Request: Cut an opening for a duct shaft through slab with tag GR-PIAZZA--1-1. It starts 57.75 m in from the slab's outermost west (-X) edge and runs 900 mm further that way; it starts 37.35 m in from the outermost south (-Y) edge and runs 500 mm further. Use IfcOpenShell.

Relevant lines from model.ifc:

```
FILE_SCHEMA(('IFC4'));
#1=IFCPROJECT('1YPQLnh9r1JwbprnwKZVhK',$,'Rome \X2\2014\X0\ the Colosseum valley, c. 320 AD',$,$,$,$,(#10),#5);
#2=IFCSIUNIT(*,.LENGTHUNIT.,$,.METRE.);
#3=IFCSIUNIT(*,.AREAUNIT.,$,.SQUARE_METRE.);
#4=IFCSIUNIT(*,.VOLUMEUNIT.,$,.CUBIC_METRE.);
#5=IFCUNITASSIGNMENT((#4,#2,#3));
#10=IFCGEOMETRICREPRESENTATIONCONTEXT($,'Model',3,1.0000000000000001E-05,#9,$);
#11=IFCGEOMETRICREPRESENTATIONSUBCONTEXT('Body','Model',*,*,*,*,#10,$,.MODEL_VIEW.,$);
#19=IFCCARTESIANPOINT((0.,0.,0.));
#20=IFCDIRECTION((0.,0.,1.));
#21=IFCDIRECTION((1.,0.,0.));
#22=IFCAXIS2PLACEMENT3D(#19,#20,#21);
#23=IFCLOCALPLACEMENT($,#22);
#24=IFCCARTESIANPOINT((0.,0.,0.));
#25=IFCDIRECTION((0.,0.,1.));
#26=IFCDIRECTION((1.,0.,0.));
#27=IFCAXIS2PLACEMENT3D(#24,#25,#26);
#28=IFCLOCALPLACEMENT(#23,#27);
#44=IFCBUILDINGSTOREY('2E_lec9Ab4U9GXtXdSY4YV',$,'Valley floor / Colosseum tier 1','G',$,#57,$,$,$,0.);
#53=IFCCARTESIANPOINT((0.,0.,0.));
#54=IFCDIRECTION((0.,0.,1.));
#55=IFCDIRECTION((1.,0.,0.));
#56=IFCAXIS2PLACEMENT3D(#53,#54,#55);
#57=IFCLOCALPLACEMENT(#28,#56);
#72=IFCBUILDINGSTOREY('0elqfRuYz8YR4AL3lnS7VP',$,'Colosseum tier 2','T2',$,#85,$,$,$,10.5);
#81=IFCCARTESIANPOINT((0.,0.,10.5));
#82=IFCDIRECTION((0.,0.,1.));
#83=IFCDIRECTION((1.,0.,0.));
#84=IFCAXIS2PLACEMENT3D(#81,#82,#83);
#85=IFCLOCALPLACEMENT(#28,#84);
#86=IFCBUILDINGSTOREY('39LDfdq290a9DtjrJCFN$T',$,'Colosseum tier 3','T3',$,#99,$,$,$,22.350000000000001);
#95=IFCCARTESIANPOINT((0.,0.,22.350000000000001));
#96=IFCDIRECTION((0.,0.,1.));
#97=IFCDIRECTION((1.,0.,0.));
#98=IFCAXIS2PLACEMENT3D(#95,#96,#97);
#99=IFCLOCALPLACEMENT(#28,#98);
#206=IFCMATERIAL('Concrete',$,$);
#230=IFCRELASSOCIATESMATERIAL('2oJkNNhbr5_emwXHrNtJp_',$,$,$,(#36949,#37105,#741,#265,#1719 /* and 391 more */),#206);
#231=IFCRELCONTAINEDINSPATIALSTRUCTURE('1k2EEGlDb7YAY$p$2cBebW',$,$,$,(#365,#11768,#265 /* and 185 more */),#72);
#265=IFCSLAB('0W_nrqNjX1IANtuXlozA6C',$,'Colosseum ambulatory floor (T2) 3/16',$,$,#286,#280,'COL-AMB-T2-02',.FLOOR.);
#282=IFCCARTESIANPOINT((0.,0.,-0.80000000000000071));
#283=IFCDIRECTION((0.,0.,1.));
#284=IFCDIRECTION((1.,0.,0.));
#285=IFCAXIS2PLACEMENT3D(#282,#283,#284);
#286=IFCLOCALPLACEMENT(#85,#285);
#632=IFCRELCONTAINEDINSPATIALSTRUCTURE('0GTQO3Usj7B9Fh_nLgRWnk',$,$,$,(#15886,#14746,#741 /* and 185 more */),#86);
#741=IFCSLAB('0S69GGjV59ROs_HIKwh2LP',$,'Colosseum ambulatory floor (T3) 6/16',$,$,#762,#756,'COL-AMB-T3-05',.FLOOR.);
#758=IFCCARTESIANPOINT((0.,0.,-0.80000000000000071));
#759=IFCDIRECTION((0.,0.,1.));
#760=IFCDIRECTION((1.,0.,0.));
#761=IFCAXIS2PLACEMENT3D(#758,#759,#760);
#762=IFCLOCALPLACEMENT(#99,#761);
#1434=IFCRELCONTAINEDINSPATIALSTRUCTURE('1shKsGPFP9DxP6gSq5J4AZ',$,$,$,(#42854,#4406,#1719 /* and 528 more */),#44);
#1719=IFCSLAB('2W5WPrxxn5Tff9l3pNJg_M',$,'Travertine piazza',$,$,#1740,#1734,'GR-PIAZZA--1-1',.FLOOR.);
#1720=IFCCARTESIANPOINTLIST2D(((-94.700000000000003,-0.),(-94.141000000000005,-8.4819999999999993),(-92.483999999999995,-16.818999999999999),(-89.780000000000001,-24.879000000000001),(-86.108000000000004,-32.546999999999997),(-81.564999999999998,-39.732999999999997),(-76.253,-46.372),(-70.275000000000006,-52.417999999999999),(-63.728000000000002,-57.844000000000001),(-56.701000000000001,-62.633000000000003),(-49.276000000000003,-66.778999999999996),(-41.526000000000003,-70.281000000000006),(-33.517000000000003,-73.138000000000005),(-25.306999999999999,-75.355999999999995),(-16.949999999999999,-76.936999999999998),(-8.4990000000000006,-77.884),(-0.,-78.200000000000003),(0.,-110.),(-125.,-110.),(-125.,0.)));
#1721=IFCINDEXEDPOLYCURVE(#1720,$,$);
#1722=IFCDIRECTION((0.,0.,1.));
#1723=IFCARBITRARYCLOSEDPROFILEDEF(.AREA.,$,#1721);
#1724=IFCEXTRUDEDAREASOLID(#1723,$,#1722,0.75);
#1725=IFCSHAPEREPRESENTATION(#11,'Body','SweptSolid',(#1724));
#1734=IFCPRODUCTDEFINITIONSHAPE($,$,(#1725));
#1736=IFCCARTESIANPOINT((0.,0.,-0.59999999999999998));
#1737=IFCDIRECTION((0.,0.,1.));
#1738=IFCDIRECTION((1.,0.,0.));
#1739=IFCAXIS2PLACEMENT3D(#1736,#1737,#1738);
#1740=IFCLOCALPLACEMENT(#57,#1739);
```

```python
import numpy as np
import ifcopenshell
import ifcopenshell.api.feature
import ifcopenshell.api.geometry
import ifcopenshell.api.root
import ifcopenshell.geom
import ifcopenshell.util.placement
import ifcopenshell.util.representation
import ifcopenshell.util.shape
import ifcopenshell.util.unit

model = ifcopenshell.open("model.ifc")
unit_scale = ifcopenshell.util.unit.calculate_unit_scale(model)
settings = ifcopenshell.geom.settings()


def volume(element):
    """Net volume in cubic metres, openings subtracted."""
    shape = ifcopenshell.geom.create_shape(settings, element)
    return ifcopenshell.util.shape.get_volume(shape.geometry)


slab = model.by_id(1719)
before = volume(slab)

# Extent in the slab's own axes, in metres. The edges named are its -X and -Y sides.
slab_shape = ifcopenshell.geom.create_shape(settings, slab)
vertices = ifcopenshell.util.shape.get_vertices(slab_shape.geometry)
x_min, y_min, bottom = vertices.min(axis=0)
top = vertices[:, 2].max()

opening = ifcopenshell.api.root.create_entity(model, ifc_class="IfcOpeningElement", name="Duct shaft opening", predefined_type="OPENING")
context = ifcopenshell.util.representation.get_context(model, "Model", "Body", "MODEL_VIEW")
width, depth = 0.9, 0.5
outline = [(0.0, 0.0), (width, 0.0), (width, depth), (0.0, depth), (0.0, 0.0)]
# Overshoot both faces by 50 mm so the cut is clean.
shape = ifcopenshell.api.geometry.add_slab_representation(
    model, context=context, depth=top - bottom + 0.1, polyline=outline
)
ifcopenshell.api.geometry.assign_representation(model, product=opening, representation=shape)

matrix = ifcopenshell.util.placement.get_local_placement(slab.ObjectPlacement)
matrix[:, 3] = matrix @ np.append(np.array([x_min + 57.75, y_min + 37.35, bottom - 0.05]) / unit_scale, 1.0)
ifcopenshell.api.geometry.edit_object_placement(model, product=opening, matrix=matrix, is_si=False)
ifcopenshell.api.feature.add_feature(model, feature=opening, element=slab)

after = volume(slab)

print(f"slab volume {before:.3f} -> {after:.3f} m3")

model.write("model_updated.ifc")
```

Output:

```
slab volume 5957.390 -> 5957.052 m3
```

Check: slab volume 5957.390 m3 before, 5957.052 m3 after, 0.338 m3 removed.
